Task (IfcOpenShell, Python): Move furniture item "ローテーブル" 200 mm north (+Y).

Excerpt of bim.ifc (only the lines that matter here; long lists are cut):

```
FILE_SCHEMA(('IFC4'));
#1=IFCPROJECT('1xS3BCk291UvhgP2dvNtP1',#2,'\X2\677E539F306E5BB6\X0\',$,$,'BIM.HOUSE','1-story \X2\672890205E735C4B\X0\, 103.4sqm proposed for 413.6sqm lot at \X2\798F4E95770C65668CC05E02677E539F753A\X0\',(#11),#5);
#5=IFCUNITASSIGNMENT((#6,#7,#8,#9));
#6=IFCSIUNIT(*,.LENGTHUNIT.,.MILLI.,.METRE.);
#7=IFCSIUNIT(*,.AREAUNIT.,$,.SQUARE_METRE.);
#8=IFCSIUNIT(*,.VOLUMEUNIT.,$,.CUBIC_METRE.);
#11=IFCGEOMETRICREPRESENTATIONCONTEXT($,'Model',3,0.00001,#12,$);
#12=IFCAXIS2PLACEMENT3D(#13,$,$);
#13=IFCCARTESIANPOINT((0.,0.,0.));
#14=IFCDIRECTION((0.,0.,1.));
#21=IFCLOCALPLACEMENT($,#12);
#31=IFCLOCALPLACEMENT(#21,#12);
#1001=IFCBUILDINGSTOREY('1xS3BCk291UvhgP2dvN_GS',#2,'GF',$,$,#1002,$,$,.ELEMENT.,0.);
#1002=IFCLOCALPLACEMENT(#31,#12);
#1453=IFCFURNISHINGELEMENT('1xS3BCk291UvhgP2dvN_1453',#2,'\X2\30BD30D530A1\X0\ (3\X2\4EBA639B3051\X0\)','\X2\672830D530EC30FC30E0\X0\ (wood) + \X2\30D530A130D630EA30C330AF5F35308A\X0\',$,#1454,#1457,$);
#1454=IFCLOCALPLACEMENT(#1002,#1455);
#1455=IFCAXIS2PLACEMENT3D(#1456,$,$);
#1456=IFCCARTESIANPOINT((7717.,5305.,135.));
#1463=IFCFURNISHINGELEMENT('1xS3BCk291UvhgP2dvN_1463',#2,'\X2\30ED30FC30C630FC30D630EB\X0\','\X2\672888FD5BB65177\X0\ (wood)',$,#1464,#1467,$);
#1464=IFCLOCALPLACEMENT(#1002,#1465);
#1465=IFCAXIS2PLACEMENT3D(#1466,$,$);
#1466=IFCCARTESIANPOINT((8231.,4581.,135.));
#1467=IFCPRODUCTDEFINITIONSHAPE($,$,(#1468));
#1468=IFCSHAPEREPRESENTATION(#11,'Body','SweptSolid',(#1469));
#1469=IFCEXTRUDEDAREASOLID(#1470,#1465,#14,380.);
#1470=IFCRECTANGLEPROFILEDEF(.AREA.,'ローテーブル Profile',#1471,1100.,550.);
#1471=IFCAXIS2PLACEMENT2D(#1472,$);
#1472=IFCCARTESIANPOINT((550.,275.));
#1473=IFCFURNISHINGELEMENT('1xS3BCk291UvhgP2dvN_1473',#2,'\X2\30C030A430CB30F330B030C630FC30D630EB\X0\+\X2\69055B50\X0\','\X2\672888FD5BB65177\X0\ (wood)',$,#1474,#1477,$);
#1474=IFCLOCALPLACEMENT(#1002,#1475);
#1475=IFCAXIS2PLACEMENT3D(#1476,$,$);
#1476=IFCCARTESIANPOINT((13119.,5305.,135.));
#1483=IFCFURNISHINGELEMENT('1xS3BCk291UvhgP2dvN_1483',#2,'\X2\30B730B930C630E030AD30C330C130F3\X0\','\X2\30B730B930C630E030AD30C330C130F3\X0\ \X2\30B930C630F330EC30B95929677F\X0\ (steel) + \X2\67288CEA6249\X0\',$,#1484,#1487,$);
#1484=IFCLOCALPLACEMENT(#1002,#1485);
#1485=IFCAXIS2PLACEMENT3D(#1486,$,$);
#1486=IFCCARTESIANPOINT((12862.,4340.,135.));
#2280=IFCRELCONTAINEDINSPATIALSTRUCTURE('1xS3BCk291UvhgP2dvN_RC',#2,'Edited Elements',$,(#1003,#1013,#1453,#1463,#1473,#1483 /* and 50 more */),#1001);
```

```python
import ifcopenshell
import ifcopenshell.api.geometry
import ifcopenshell.util.placement
import ifcopenshell.util.unit

model = ifcopenshell.open("bim.ifc")
unit_scale = ifcopenshell.util.unit.calculate_unit_scale(model)

item = model.by_guid("1xS3BCk291UvhgP2dvN_1463")
matrix = ifcopenshell.util.placement.get_local_placement(item.ObjectPlacement)
matrix[1, 3] += 0.2 / unit_scale
ifcopenshell.api.geometry.edit_object_placement(model, product=item, matrix=matrix, is_si=False)

print(ifcopenshell.util.placement.get_local_placement(item.ObjectPlacement).round(3) + 0.0)

model.write("bim_v2.ifc")
```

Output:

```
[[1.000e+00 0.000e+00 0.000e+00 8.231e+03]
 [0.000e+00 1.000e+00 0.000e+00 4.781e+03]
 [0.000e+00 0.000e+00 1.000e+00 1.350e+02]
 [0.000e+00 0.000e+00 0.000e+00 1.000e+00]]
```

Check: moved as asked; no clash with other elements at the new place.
